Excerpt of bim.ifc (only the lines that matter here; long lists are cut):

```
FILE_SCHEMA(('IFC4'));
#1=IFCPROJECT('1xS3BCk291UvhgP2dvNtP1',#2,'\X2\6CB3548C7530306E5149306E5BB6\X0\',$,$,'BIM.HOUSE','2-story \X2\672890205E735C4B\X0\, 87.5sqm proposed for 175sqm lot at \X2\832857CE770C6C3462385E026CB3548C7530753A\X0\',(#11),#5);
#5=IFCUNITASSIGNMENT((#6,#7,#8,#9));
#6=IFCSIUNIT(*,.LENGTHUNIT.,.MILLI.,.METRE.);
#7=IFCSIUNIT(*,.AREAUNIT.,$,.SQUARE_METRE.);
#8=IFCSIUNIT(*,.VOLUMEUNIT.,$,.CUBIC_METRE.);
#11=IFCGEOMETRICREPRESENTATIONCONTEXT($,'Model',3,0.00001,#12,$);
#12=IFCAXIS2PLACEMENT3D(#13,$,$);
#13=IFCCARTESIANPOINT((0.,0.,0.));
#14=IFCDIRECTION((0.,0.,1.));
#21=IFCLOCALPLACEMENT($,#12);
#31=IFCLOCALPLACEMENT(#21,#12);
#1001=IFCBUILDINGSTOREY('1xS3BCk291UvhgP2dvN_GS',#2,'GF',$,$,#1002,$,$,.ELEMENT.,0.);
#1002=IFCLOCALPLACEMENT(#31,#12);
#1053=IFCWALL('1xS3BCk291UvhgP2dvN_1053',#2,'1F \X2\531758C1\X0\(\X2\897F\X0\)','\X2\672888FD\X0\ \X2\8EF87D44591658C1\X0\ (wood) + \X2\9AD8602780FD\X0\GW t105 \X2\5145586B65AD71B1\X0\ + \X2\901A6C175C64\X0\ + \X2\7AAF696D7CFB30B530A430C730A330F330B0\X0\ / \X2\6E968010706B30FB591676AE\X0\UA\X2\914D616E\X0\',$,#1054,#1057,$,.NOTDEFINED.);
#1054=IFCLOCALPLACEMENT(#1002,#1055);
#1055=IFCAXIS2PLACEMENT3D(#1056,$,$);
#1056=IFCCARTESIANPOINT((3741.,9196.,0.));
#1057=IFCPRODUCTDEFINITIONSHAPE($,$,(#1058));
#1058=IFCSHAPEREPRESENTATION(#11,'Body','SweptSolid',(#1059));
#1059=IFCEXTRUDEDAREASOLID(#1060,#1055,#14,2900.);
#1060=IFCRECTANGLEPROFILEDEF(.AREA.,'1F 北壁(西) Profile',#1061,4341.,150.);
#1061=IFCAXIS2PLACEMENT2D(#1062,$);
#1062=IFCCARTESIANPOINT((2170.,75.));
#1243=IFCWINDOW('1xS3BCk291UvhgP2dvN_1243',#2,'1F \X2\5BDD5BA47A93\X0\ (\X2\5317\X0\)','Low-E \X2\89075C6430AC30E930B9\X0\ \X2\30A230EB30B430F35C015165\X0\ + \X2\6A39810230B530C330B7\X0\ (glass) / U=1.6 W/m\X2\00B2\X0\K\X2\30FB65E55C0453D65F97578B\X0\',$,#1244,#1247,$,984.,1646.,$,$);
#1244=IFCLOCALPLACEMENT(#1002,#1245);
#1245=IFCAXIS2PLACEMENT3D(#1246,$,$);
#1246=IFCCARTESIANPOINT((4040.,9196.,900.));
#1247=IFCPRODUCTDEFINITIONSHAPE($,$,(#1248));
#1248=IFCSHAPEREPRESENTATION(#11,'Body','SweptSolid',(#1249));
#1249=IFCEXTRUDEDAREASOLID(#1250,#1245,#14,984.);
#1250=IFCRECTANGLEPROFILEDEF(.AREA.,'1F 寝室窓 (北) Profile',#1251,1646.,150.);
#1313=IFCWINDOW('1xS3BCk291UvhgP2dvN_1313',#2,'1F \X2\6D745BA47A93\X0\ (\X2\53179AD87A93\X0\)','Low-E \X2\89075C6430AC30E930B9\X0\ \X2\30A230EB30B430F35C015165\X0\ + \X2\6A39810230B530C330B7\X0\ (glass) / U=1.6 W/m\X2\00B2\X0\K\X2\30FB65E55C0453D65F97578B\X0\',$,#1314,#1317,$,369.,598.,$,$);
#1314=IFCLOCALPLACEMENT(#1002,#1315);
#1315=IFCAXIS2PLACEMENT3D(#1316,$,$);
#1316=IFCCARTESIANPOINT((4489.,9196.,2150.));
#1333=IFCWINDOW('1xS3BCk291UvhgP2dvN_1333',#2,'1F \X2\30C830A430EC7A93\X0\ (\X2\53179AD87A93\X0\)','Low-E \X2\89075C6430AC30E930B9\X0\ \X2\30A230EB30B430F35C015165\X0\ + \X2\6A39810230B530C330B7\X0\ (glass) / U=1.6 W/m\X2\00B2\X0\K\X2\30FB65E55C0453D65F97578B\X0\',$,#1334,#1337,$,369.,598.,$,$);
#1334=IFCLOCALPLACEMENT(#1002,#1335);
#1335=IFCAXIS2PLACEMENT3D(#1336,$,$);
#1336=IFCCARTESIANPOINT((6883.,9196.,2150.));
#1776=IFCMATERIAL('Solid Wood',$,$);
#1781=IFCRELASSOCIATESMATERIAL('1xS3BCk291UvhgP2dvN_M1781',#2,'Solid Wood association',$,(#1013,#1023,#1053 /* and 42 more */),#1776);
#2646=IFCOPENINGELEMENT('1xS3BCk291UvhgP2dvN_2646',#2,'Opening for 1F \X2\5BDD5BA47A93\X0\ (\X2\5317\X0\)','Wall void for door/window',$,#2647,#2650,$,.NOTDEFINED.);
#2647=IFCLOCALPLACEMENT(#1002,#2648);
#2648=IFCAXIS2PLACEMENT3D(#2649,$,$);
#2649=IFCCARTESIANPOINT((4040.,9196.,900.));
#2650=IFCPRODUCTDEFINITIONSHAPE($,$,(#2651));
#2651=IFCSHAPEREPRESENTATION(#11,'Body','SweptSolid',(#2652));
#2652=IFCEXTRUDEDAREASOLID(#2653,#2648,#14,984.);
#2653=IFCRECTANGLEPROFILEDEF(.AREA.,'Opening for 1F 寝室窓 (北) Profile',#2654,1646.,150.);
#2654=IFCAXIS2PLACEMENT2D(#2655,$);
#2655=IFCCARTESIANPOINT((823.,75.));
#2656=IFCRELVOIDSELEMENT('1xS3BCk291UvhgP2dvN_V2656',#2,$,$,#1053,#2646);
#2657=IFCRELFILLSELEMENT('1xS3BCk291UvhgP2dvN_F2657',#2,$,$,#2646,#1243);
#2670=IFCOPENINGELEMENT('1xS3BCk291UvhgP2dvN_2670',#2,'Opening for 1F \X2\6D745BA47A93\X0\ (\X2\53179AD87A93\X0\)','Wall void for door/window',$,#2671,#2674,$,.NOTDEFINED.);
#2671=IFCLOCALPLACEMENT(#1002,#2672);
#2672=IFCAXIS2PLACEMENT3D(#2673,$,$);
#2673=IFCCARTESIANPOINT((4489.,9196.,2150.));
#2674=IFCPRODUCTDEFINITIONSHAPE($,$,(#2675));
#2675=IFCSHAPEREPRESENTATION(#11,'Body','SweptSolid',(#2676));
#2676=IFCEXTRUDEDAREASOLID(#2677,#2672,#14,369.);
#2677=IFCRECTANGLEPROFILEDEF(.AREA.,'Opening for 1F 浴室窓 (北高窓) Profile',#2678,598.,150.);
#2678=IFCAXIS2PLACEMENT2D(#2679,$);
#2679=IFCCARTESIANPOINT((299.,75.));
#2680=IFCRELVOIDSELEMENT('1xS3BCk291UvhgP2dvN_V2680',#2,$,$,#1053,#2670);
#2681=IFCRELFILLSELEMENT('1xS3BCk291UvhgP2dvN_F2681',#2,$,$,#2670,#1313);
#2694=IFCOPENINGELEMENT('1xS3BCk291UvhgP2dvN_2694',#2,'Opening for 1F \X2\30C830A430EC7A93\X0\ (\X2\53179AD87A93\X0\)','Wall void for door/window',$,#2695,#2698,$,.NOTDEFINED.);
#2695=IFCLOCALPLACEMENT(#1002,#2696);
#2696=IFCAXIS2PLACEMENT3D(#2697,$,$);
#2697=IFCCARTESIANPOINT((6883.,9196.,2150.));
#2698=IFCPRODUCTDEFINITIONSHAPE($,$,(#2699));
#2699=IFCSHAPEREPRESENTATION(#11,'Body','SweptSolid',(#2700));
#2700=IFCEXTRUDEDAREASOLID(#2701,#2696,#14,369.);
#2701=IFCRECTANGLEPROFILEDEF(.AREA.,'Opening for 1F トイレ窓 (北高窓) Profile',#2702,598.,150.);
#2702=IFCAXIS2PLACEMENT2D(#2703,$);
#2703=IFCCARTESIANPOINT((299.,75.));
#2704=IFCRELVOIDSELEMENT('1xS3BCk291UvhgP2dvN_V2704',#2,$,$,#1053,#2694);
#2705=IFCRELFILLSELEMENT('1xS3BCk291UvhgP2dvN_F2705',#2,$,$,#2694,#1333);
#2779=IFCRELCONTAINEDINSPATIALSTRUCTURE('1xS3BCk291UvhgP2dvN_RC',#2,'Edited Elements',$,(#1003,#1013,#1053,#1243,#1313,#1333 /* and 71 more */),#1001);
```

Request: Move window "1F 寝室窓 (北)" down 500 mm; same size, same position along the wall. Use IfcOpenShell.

```python
import numpy as np
import ifcopenshell
import ifcopenshell.api.geometry
import ifcopenshell.util.placement
import ifcopenshell.util.unit

model = ifcopenshell.open("bim.ifc")
unit_scale = ifcopenshell.util.unit.calculate_unit_scale(model)

window = model.by_guid("1xS3BCk291UvhgP2dvN_1243")
opening = window.FillsVoids[0].RelatingOpeningElement
dz = -0.5 / unit_scale

shift = np.array([0.0, 0.0, dz])
# The window is not placed relative to its opening, so move both.
for product in (opening, window):
    matrix = ifcopenshell.util.placement.get_local_placement(product.ObjectPlacement)
    matrix[:3, 3] += shift
    ifcopenshell.api.geometry.edit_object_placement(model, product=product, matrix=matrix, is_si=False)

print(f"moved by {dz * unit_scale:+.3f} m")

model.write("bim_rev.ifc")
```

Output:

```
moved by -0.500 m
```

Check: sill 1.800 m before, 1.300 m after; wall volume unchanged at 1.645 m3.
